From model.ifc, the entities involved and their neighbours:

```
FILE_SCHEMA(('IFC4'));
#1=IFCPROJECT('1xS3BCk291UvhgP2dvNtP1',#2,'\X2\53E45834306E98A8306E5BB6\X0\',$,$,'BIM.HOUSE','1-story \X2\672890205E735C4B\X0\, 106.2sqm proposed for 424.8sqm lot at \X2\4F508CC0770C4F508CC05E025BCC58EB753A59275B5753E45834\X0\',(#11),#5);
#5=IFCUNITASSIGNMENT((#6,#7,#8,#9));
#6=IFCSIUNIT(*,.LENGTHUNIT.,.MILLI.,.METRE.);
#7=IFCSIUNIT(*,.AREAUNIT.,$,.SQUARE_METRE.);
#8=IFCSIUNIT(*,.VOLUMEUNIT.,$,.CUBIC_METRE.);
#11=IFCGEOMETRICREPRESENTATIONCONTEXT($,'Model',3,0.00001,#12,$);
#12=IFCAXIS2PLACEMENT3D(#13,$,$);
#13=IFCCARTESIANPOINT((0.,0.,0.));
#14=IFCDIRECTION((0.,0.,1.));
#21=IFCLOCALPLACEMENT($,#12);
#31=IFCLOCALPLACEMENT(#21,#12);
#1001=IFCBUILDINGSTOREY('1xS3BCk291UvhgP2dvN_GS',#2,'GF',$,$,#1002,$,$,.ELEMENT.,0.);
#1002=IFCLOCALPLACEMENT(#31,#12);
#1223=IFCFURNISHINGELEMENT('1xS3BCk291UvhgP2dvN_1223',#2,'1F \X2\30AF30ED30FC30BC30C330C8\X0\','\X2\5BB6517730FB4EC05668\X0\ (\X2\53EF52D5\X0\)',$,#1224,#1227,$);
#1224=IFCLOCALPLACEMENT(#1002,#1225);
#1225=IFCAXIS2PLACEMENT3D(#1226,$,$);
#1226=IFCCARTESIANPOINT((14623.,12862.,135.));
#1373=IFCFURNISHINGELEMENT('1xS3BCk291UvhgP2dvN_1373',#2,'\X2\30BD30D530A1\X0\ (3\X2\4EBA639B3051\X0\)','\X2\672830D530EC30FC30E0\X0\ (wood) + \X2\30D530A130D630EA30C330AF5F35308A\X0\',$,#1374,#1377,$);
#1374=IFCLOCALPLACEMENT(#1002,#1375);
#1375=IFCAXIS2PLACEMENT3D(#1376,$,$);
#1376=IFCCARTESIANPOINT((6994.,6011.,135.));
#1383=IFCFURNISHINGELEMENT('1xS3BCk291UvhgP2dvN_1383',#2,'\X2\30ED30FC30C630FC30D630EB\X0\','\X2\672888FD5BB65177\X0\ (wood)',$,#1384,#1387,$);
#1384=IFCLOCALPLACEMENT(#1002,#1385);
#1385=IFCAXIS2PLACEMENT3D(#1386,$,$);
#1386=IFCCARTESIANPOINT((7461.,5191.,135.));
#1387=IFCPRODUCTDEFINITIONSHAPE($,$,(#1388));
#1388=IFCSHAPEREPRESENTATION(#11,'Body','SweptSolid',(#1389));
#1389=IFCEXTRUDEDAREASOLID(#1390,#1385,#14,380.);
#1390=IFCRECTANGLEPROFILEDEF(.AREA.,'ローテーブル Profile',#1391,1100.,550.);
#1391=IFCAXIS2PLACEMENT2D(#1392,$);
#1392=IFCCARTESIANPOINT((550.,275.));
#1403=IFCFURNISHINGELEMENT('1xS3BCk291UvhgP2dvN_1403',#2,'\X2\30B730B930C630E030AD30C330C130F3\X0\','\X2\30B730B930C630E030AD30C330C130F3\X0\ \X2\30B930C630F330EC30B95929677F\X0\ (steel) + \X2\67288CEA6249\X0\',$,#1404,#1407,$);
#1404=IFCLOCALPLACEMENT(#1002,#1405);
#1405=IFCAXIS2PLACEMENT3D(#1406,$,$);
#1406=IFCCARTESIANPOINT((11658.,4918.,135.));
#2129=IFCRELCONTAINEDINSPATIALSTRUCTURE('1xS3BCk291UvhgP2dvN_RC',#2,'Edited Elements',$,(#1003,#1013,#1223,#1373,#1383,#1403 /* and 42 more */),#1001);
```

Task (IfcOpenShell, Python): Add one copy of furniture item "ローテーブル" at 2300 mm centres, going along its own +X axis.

```python
import ifcopenshell
import ifcopenshell.api.geometry
import ifcopenshell.api.root
import ifcopenshell.util.element
import ifcopenshell.util.placement
import ifcopenshell.util.unit

model = ifcopenshell.open("model.ifc")
unit_scale = ifcopenshell.util.unit.calculate_unit_scale(model)


def reuse_history(source, copy):
    """copy_class also copies each property set's owner history, people and application; keep the originals."""
    for rel in copy.IsDefinedBy:
        if rel.is_a("IfcRelDefinesByProperties") and (history := rel.RelatingPropertyDefinition.OwnerHistory):
            rel.RelatingPropertyDefinition.OwnerHistory = source.OwnerHistory
            ifcopenshell.util.element.remove_deep2(model, history)


source = model.by_guid("1xS3BCk291UvhgP2dvN_1383")
base = ifcopenshell.util.placement.get_local_placement(source.ObjectPlacement)
step = base[:3, 0] * 2.3 / unit_scale

for i in range(1, 2):
    copy = ifcopenshell.api.root.copy_class(model, product=source)
    copy.Representation = ifcopenshell.util.element.copy_deep(
        model, source.Representation, exclude=["IfcGeometricRepresentationContext", "IfcRepresentationMap"]
    )
    reuse_history(source, copy)
    matrix = base.copy()
    matrix[:3, 3] += i * step
    print("added at", matrix[:3, 3].round(3) + 0.0)
    ifcopenshell.api.geometry.edit_object_placement(model, product=copy, matrix=matrix, is_si=False)

model.write("model_edited.ifc")
```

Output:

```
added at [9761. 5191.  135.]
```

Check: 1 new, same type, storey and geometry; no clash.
